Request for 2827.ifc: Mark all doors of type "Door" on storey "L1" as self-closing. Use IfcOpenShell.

First a look at what the model holds.

```python
import ifcopenshell
import ifcopenshell.util.element

model = ifcopenshell.open("2827.ifc")
print(model.schema)
storey = next(s for s in model.by_type("IfcBuildingStorey") if s.Name == "L1")
doors = [e for e in ifcopenshell.util.element.get_decomposition(storey) if e.is_a("IfcDoor")]
seen = {}
for e in doors:
    element_type = ifcopenshell.util.element.get_type(e)
    key = (element_type.Name if element_type != e and element_type else None, ifcopenshell.util.element.get_pset(e, "Pset_DoorCommon", "SelfClosing"))
    seen[key] = seen.get(key, 0) + 1
for (name, value), count in sorted(seen.items(), key=str):
    print(count, "x", name, "|", value)
```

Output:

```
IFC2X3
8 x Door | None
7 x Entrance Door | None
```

```python
import ifcopenshell
import ifcopenshell.api.pset
import ifcopenshell.util.element

model = ifcopenshell.open("2827.ifc")

storey = next(s for s in model.by_type("IfcBuildingStorey") if s.Name == "L1")
doors = [e for e in ifcopenshell.util.element.get_decomposition(storey) if e.is_a("IfcDoor")]

count = 0
for e in doors:
    element_type = ifcopenshell.util.element.get_type(e)
    if element_type in (None, e) or element_type.Name != "Door":
        continue
    # add_pset returns the element's existing set when there is one.
    pset = ifcopenshell.api.pset.add_pset(model, product=e, name="Pset_DoorCommon")
    ifcopenshell.api.pset.edit_pset(model, pset=pset, properties={"SelfClosing": True})
    count += 1

print(count, "doors updated")

model.write("2827_rev.ifc")
```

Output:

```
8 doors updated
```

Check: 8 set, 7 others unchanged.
